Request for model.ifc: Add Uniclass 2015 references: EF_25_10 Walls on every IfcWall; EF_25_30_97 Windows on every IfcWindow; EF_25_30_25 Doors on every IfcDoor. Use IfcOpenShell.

First a look at what the model holds.

```python
import ifcopenshell

model = ifcopenshell.open("model.ifc")
print(model.schema)
print("classifications:", [c.Name for c in model.by_type("IfcClassification")])
for ifc_class in ("IfcDoor", "IfcRoof", "IfcStair", "IfcWall", "IfcWindow"):
    print(ifc_class, len(model.by_type(ifc_class)))
```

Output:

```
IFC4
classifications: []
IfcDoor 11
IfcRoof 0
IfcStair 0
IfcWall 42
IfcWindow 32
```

```python
import ifcopenshell
import ifcopenshell.api.classification

model = ifcopenshell.open("model.ifc")

system = ifcopenshell.api.classification.add_classification(model, classification="Uniclass 2015")

codes = {
    "IfcWall": ("EF_25_10", "Walls"),
    "IfcWindow": ("EF_25_30_97", "Windows"),
    "IfcDoor": ("EF_25_30_25", "Doors"),
}
for ifc_class, (code, name) in codes.items():
    products = model.by_type(ifc_class)
    ifcopenshell.api.classification.add_reference(
        model, products=products, classification=system, identification=code, name=name
    )
    print(code, len(products))

model.write("model-out.ifc")
```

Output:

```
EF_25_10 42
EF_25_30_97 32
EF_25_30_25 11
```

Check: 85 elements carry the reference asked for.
